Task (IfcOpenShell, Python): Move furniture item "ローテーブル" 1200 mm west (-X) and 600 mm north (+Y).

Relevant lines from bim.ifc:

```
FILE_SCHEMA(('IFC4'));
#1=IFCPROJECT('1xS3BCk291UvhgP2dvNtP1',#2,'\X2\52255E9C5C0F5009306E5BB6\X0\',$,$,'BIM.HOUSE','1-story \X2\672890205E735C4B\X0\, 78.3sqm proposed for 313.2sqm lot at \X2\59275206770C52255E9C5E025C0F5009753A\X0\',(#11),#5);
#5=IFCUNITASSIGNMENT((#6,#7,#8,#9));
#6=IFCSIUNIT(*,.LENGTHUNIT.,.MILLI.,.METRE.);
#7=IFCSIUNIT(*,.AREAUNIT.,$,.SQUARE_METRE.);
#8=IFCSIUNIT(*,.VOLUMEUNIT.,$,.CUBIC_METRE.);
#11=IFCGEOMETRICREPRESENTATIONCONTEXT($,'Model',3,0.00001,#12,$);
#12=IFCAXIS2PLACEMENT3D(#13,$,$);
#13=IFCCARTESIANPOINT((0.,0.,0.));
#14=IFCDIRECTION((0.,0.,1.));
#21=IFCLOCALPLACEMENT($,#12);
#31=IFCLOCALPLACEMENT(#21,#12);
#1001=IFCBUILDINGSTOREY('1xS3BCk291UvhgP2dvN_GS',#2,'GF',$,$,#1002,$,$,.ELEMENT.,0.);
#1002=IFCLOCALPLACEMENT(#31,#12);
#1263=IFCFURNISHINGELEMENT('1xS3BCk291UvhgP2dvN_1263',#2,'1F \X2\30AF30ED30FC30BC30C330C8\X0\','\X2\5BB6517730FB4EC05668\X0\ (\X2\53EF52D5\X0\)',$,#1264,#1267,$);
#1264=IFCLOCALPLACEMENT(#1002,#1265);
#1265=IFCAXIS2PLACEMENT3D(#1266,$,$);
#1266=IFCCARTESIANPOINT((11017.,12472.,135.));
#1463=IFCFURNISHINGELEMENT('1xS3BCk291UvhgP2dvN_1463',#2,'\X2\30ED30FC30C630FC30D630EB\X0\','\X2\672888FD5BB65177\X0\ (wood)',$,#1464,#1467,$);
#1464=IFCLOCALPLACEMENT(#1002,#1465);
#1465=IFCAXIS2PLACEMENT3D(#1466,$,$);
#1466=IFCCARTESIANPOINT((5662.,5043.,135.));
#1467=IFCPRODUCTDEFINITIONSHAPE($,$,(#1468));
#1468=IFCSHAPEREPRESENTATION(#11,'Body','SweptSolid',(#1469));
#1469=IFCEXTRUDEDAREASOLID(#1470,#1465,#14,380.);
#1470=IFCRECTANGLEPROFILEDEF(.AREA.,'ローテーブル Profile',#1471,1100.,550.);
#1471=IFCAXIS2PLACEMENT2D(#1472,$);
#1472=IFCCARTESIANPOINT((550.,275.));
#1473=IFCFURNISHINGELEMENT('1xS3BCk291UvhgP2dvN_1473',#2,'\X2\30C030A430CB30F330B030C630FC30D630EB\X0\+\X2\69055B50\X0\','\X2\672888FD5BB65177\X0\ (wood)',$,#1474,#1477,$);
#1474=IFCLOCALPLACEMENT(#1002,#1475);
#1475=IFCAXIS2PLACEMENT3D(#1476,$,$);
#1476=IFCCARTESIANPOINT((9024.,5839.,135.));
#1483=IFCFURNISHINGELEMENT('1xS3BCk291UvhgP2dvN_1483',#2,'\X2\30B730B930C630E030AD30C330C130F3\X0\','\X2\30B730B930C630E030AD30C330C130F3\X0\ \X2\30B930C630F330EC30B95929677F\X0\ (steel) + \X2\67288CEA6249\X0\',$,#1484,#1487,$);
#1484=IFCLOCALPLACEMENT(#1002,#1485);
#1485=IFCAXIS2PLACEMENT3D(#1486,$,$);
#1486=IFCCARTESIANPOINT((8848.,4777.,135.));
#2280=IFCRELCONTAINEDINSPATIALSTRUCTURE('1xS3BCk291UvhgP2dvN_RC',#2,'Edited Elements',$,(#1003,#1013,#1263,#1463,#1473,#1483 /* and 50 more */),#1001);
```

```python
import ifcopenshell
import ifcopenshell.api.geometry
import ifcopenshell.util.placement
import ifcopenshell.util.unit

model = ifcopenshell.open("bim.ifc")
unit_scale = ifcopenshell.util.unit.calculate_unit_scale(model)

item = model.by_guid("1xS3BCk291UvhgP2dvN_1463")
matrix = ifcopenshell.util.placement.get_local_placement(item.ObjectPlacement)
matrix[0, 3] -= 1.2 / unit_scale
matrix[1, 3] += 0.6 / unit_scale
ifcopenshell.api.geometry.edit_object_placement(model, product=item, matrix=matrix, is_si=False)

print(ifcopenshell.util.placement.get_local_placement(item.ObjectPlacement).round(3) + 0.0)

model.write("bim-out.ifc")
```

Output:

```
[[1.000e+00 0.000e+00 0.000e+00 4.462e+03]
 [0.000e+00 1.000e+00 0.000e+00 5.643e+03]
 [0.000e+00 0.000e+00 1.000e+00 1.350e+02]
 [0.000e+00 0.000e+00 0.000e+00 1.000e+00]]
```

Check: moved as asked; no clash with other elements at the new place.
